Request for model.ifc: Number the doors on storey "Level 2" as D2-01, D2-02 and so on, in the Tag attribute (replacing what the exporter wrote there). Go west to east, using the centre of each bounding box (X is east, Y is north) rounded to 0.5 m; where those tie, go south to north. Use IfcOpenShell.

First a look at what the model holds.

```python
import ifcopenshell
import ifcopenshell.util.element
import ifcopenshell.util.placement

model = ifcopenshell.open("model.ifc")
print(model.schema)
storey = next(s for s in model.by_type("IfcBuildingStorey") if s.Name == "Level 2")
doors = [e for e in ifcopenshell.util.element.get_decomposition(storey) if e.is_a("IfcDoor")]
for e in sorted(doors, key=lambda e: e.id()):
    origin = ifcopenshell.util.placement.get_local_placement(e.ObjectPlacement)[:3, 3]
    print(e.id(), e.Tag, e.Name, origin.round(2) + 0.0, sep=" | ")
```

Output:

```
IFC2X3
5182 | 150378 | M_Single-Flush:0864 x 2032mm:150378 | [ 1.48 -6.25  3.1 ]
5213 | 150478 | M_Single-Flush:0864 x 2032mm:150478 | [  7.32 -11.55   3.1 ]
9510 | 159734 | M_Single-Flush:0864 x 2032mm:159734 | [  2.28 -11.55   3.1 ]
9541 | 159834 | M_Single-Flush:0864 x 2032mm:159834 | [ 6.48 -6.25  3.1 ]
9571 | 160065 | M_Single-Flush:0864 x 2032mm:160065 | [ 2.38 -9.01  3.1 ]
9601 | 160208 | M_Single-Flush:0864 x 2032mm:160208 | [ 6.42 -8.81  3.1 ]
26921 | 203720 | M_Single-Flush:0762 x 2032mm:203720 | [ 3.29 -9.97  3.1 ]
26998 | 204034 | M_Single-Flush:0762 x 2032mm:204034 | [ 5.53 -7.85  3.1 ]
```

```python
import ifcopenshell
import ifcopenshell.geom
import ifcopenshell.util.element
import ifcopenshell.util.shape

model = ifcopenshell.open("model.ifc")
settings = ifcopenshell.geom.settings()
settings.set("use-world-coords", True)


def centre(element):
    shape = ifcopenshell.geom.create_shape(settings, element)
    return ifcopenshell.util.shape.get_bbox_centroid(shape.geometry)


storey = next(s for s in model.by_type("IfcBuildingStorey") if s.Name == "Level 2")
doors = [e for e in ifcopenshell.util.element.get_decomposition(storey) if e.is_a("IfcDoor")]

# Insertion points can sit at a corner or the storey origin, so sort by the geometry (in metres).
centres = {e: centre(e) for e in doors}
doors.sort(key=lambda e: (round(centres[e][0] / 0.5), centres[e][1]))

for i, e in enumerate(doors, start=1):
    number = f"D2-{i:02d}"
    e.Tag = number
    print(e.id(), number)

model.write("model-out.ifc")
```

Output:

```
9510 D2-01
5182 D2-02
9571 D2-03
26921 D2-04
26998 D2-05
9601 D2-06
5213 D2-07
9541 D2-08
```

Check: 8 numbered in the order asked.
